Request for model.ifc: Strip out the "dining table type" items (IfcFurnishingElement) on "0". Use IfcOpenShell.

First a look at what the model holds.

```python
import ifcopenshell
import ifcopenshell.util.element

model = ifcopenshell.open("model.ifc")
print(model.schema)
storey = next(s for s in model.by_type("IfcBuildingStorey") if s.Name == "0")
furniture = [e for e in ifcopenshell.util.element.get_decomposition(storey) if e.is_a("IfcFurnishingElement")]
seen = {}
for e in furniture:
    element_type = ifcopenshell.util.element.get_type(e)
    name = element_type.Name if element_type not in (None, e) else None
    seen[name] = seen.get(name, 0) + 1
for name, count in sorted(seen.items(), key=str):
    print(count, "x", name)
```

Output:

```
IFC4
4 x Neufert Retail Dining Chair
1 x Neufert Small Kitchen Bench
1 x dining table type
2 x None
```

```python
import ifcopenshell
import ifcopenshell.api.root
import ifcopenshell.util.element

model = ifcopenshell.open("model.ifc")

storey = next(s for s in model.by_type("IfcBuildingStorey") if s.Name == "0")
furniture = [e for e in ifcopenshell.util.element.get_decomposition(storey) if e.is_a("IfcFurnishingElement")]
targets = [e for e in furniture if (t := ifcopenshell.util.element.get_type(e)) not in (None, e) and t.Name == "dining table type"]

for e in targets:
    ifcopenshell.api.root.remove_product(model, product=e)
print(len(targets), "removed")

model.write("model_updated.ifc")
```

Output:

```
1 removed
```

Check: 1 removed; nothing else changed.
